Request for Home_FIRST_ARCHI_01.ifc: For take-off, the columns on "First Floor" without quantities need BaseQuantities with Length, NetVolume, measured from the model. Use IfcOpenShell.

First a look at what the model holds.

```python
import ifcopenshell
import ifcopenshell.util.element
import ifcopenshell.util.unit

model = ifcopenshell.open("Home_FIRST_ARCHI_01.ifc")
print(model.schema)
for unit_type in ("LENGTHUNIT", "AREAUNIT", "VOLUMEUNIT"):
    print(unit_type, ifcopenshell.util.unit.calculate_unit_scale(model, unit_type))
storey = next(s for s in model.by_type("IfcBuildingStorey") if s.Name == "First Floor")
columns = [e for e in ifcopenshell.util.element.get_decomposition(storey) if e.is_a("IfcColumn")]
for e in sorted(columns, key=lambda e: e.id()):
    print(e.id(), e.is_a(), e.Name, list(ifcopenshell.util.element.get_psets(e, qtos_only=True)), sep=" | ")
```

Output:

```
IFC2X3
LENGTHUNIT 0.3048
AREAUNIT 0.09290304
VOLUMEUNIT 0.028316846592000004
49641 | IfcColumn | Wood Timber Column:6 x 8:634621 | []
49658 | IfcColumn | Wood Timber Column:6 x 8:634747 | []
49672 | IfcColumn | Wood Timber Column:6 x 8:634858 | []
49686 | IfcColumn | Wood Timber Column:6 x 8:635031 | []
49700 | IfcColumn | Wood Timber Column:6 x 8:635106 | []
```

```python
import ifcopenshell
import ifcopenshell.api.pset
import ifcopenshell.geom
import ifcopenshell.util.element
import ifcopenshell.util.shape
import ifcopenshell.util.unit

model = ifcopenshell.open("Home_FIRST_ARCHI_01.ifc")
unit_scale = ifcopenshell.util.unit.calculate_unit_scale(model)
volume_scale = ifcopenshell.util.unit.calculate_unit_scale(model, "VOLUMEUNIT")
settings = ifcopenshell.geom.settings()

storey = next(s for s in model.by_type("IfcBuildingStorey") if s.Name == "First Floor")
columns = [e for e in ifcopenshell.util.element.get_decomposition(storey) if e.is_a("IfcColumn")]

for e in sorted(columns, key=lambda e: e.id()):
    if ifcopenshell.util.element.get_psets(e, qtos_only=True, should_inherit=False):
        continue
    # Geometry comes back in metres, in the element's own axes.
    shape = ifcopenshell.geom.create_shape(settings, e)
    values = {
        "Length": ifcopenshell.util.shape.get_z(shape.geometry) / unit_scale,
        "NetVolume": ifcopenshell.util.shape.get_volume(shape.geometry) / volume_scale,
    }
    qto = ifcopenshell.api.pset.add_qto(model, product=e, name="BaseQuantities")
    ifcopenshell.api.pset.edit_qto(model, qto=qto, properties=values)
    print(e.id(), {k: round(v, 3) for k, v in values.items()})

model.write("Home_FIRST_ARCHI_01_edited.ifc")
```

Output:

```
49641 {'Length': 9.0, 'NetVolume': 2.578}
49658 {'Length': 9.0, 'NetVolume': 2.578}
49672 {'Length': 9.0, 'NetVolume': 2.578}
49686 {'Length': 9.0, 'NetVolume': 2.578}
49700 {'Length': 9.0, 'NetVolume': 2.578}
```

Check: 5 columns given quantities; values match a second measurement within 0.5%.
